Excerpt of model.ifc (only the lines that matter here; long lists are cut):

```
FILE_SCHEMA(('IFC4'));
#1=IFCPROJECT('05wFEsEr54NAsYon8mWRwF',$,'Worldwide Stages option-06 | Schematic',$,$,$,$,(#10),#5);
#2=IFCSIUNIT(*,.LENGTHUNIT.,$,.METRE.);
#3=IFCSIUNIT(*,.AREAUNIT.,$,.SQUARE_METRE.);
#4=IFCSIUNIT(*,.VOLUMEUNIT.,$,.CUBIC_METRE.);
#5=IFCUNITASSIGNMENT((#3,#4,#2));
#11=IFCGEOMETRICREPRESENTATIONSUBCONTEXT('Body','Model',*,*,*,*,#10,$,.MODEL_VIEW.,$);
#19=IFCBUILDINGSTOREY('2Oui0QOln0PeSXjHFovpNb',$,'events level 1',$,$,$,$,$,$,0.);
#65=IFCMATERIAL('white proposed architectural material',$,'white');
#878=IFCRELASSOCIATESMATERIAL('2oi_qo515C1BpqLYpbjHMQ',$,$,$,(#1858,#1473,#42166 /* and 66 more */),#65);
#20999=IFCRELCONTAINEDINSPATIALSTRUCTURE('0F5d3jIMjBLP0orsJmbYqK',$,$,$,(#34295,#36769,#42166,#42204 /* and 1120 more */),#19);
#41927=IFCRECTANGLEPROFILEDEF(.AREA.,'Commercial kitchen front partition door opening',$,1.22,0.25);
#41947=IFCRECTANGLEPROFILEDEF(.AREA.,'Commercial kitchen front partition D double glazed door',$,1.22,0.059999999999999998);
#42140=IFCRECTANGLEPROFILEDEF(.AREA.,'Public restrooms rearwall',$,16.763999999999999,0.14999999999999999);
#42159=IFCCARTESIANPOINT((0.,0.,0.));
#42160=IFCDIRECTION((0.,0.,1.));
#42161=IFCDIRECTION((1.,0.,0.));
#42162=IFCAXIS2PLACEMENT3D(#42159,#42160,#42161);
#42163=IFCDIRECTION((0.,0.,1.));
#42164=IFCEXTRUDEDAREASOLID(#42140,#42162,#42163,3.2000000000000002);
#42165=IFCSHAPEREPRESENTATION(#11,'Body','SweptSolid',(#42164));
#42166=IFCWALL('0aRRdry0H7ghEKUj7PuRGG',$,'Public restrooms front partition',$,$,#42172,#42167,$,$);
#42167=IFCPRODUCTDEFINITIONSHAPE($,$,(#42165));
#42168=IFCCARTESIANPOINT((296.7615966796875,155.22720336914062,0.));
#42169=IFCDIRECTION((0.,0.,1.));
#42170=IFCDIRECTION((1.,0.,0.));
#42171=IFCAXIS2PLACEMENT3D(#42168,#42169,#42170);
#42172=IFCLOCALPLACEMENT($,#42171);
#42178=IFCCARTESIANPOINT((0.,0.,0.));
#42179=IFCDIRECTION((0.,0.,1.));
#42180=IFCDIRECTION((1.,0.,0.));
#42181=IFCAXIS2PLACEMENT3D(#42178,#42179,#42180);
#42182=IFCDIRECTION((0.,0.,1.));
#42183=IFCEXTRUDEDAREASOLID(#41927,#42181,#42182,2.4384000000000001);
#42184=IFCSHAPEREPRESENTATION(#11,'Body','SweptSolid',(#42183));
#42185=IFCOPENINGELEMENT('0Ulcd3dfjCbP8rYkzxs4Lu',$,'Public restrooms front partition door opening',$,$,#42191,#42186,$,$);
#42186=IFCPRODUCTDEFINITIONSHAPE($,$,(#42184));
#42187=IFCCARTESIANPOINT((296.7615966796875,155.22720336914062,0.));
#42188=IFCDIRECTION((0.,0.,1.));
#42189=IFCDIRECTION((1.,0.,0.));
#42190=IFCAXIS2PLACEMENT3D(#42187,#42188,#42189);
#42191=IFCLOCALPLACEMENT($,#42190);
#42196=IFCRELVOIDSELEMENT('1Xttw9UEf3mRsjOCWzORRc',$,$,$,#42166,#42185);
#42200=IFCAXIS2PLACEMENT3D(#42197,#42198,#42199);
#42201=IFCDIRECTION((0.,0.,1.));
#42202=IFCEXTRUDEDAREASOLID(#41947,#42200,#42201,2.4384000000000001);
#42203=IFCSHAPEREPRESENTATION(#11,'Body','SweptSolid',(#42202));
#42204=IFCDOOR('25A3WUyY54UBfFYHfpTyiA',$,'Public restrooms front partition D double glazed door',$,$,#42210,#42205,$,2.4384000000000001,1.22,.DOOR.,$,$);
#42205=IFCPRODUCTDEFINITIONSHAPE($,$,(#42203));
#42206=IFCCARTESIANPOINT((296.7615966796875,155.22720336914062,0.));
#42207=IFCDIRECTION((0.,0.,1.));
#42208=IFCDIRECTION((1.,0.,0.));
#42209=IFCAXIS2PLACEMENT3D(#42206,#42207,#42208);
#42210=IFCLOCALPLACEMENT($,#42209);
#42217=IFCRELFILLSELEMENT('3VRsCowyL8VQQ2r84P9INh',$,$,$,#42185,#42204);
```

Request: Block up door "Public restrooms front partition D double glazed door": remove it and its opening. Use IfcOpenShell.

```python
import ifcopenshell
import ifcopenshell.api.feature
import ifcopenshell.api.root
import ifcopenshell.geom
import ifcopenshell.util.shape

model = ifcopenshell.open("model.ifc")
settings = ifcopenshell.geom.settings()


def volume(element):
    """Net volume in cubic metres, openings subtracted."""
    shape = ifcopenshell.geom.create_shape(settings, element)
    return ifcopenshell.util.shape.get_volume(shape.geometry)


door = model.by_guid("25A3WUyY54UBfFYHfpTyiA")
opening = door.FillsVoids[0].RelatingOpeningElement
wall = opening.VoidsElements[0].RelatingBuildingElement
before = volume(wall)

ifcopenshell.api.root.remove_product(model, product=door)
ifcopenshell.api.feature.remove_feature(model, feature=opening)

after = volume(wall)

print(f"wall volume {before:.3f} -> {after:.3f} m3")

model.write("model_updated.ifc")
```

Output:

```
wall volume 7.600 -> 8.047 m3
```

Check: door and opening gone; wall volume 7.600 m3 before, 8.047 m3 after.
